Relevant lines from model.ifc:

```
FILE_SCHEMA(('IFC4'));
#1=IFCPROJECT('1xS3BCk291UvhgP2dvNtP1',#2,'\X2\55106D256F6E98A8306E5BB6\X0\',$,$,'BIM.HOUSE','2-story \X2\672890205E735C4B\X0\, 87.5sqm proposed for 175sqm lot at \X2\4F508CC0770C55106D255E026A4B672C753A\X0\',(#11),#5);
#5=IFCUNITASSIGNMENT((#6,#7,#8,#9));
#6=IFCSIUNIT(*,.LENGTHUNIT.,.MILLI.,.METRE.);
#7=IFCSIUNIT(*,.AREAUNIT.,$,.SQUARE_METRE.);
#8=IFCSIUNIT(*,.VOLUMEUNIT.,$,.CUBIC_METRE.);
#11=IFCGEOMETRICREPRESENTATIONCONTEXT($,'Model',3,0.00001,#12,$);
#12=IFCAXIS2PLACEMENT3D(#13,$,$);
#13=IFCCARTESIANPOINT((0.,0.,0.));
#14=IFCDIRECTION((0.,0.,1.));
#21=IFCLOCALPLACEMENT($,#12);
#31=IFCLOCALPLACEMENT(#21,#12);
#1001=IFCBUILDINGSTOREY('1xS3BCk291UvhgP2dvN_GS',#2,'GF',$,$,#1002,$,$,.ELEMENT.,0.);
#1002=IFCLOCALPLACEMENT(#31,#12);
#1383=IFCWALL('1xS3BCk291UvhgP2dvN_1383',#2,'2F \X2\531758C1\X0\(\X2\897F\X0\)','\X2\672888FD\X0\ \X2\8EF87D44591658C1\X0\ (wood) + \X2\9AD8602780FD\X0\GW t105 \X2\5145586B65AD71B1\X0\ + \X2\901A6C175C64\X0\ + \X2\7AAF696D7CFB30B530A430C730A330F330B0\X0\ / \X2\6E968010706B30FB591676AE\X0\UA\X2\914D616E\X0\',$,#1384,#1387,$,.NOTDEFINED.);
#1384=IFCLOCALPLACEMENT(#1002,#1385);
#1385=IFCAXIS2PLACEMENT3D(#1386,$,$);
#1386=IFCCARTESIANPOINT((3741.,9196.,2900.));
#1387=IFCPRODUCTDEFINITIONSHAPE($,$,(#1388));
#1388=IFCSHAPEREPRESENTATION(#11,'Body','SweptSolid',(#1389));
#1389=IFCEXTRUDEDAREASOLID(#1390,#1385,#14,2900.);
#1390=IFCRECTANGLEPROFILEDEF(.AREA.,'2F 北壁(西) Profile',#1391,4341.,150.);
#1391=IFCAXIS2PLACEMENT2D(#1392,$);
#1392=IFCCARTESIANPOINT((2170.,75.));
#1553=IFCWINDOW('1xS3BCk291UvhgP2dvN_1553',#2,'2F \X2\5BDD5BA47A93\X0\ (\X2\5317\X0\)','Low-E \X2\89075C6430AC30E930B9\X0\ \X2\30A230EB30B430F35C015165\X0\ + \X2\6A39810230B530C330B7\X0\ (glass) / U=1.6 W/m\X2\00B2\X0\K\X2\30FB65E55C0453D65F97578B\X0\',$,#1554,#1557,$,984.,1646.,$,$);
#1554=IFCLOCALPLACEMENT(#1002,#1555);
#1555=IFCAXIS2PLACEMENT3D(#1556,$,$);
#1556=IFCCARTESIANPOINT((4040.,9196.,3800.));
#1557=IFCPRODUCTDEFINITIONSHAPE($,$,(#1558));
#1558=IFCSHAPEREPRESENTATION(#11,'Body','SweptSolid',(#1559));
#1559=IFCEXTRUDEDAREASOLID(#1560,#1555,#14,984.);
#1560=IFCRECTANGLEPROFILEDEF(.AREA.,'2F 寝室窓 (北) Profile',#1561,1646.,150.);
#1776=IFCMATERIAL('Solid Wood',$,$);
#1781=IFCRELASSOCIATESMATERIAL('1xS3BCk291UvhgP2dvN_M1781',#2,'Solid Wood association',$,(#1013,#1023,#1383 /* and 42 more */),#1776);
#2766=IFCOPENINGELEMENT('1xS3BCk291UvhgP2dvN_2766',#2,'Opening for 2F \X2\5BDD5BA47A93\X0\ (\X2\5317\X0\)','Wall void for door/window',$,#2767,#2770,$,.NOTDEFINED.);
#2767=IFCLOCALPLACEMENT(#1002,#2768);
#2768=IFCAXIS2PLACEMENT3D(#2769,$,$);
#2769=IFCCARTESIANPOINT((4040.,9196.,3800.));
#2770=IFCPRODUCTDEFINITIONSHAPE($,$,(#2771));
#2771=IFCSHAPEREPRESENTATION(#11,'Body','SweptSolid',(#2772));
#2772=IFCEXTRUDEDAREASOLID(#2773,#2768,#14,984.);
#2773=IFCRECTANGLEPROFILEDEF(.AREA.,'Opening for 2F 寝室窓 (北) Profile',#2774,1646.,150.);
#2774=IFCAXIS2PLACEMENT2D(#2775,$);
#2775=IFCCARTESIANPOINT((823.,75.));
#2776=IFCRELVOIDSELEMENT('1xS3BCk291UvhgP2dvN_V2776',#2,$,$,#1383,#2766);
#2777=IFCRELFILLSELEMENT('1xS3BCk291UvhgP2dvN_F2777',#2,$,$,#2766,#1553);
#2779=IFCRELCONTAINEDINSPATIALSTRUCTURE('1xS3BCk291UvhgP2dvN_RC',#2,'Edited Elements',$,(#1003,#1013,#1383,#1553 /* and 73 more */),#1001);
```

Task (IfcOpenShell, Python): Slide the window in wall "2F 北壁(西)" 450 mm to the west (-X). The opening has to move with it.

```python
import ifcopenshell
import ifcopenshell.api.geometry
import ifcopenshell.util.placement

model = ifcopenshell.open("model.ifc")

window = model.by_guid("1xS3BCk291UvhgP2dvN_1553")
opening = window.FillsVoids[0].RelatingOpeningElement
wall = opening.VoidsElements[0].RelatingBuildingElement

wall_matrix = ifcopenshell.util.placement.get_local_placement(wall.ObjectPlacement)
shift = wall_matrix[:3, 0] * -450.0
before = ifcopenshell.util.placement.get_local_placement(window.ObjectPlacement)[:3, 3].copy()

# The window is not placed relative to its opening, so move both.
for product in (opening, window):
    matrix = ifcopenshell.util.placement.get_local_placement(product.ObjectPlacement)
    matrix[:3, 3] += shift
    ifcopenshell.api.geometry.edit_object_placement(model, product=product, matrix=matrix, is_si=False)

after = ifcopenshell.util.placement.get_local_placement(window.ObjectPlacement)[:3, 3]
print("window moved by", (after - before).round(3) + 0.0)

model.write("model_v2.ifc")
```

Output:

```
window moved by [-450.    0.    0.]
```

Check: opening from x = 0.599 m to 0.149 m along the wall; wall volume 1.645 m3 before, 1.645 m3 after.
